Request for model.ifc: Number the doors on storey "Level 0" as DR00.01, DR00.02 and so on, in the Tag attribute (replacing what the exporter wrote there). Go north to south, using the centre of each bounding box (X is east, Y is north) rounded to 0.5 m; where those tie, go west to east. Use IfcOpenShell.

First a look at what the model holds.

```python
import ifcopenshell
import ifcopenshell.util.element
import ifcopenshell.util.placement

model = ifcopenshell.open("model.ifc")
print(model.schema)
storey = next(s for s in model.by_type("IfcBuildingStorey") if s.Name == "Level 0")
doors = [e for e in ifcopenshell.util.element.get_decomposition(storey) if e.is_a("IfcDoor")]
for e in sorted(doors, key=lambda e: e.id()):
    origin = ifcopenshell.util.placement.get_local_placement(e.ObjectPlacement)[:3, 3]
    print(e.id(), e.Tag, e.Name, origin.round(2) + 0.0, sep=" | ")
```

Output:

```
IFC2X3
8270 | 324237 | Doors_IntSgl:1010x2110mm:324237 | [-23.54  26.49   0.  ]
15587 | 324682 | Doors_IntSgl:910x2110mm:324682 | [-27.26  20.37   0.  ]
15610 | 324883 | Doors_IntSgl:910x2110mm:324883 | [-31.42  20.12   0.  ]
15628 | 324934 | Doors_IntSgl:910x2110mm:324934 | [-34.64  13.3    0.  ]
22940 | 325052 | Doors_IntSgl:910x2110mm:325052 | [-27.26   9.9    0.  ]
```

```python
import ifcopenshell
import ifcopenshell.geom
import ifcopenshell.util.element
import ifcopenshell.util.shape

model = ifcopenshell.open("model.ifc")
settings = ifcopenshell.geom.settings()
settings.set("use-world-coords", True)


def centre(element):
    shape = ifcopenshell.geom.create_shape(settings, element)
    return ifcopenshell.util.shape.get_bbox_centroid(shape.geometry)


storey = next(s for s in model.by_type("IfcBuildingStorey") if s.Name == "Level 0")
doors = [e for e in ifcopenshell.util.element.get_decomposition(storey) if e.is_a("IfcDoor")]

# Insertion points can sit at a corner or the storey origin, so sort by the geometry (in metres).
centres = {e: centre(e) for e in doors}
doors.sort(key=lambda e: (-round(centres[e][1] / 0.5), centres[e][0]))

for i, e in enumerate(doors, start=1):
    number = f"DR00.{i:02d}"
    e.Tag = number
    print(e.id(), number)

model.write("model_updated.ifc")
```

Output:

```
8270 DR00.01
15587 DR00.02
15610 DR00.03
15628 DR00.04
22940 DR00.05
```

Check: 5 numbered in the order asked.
